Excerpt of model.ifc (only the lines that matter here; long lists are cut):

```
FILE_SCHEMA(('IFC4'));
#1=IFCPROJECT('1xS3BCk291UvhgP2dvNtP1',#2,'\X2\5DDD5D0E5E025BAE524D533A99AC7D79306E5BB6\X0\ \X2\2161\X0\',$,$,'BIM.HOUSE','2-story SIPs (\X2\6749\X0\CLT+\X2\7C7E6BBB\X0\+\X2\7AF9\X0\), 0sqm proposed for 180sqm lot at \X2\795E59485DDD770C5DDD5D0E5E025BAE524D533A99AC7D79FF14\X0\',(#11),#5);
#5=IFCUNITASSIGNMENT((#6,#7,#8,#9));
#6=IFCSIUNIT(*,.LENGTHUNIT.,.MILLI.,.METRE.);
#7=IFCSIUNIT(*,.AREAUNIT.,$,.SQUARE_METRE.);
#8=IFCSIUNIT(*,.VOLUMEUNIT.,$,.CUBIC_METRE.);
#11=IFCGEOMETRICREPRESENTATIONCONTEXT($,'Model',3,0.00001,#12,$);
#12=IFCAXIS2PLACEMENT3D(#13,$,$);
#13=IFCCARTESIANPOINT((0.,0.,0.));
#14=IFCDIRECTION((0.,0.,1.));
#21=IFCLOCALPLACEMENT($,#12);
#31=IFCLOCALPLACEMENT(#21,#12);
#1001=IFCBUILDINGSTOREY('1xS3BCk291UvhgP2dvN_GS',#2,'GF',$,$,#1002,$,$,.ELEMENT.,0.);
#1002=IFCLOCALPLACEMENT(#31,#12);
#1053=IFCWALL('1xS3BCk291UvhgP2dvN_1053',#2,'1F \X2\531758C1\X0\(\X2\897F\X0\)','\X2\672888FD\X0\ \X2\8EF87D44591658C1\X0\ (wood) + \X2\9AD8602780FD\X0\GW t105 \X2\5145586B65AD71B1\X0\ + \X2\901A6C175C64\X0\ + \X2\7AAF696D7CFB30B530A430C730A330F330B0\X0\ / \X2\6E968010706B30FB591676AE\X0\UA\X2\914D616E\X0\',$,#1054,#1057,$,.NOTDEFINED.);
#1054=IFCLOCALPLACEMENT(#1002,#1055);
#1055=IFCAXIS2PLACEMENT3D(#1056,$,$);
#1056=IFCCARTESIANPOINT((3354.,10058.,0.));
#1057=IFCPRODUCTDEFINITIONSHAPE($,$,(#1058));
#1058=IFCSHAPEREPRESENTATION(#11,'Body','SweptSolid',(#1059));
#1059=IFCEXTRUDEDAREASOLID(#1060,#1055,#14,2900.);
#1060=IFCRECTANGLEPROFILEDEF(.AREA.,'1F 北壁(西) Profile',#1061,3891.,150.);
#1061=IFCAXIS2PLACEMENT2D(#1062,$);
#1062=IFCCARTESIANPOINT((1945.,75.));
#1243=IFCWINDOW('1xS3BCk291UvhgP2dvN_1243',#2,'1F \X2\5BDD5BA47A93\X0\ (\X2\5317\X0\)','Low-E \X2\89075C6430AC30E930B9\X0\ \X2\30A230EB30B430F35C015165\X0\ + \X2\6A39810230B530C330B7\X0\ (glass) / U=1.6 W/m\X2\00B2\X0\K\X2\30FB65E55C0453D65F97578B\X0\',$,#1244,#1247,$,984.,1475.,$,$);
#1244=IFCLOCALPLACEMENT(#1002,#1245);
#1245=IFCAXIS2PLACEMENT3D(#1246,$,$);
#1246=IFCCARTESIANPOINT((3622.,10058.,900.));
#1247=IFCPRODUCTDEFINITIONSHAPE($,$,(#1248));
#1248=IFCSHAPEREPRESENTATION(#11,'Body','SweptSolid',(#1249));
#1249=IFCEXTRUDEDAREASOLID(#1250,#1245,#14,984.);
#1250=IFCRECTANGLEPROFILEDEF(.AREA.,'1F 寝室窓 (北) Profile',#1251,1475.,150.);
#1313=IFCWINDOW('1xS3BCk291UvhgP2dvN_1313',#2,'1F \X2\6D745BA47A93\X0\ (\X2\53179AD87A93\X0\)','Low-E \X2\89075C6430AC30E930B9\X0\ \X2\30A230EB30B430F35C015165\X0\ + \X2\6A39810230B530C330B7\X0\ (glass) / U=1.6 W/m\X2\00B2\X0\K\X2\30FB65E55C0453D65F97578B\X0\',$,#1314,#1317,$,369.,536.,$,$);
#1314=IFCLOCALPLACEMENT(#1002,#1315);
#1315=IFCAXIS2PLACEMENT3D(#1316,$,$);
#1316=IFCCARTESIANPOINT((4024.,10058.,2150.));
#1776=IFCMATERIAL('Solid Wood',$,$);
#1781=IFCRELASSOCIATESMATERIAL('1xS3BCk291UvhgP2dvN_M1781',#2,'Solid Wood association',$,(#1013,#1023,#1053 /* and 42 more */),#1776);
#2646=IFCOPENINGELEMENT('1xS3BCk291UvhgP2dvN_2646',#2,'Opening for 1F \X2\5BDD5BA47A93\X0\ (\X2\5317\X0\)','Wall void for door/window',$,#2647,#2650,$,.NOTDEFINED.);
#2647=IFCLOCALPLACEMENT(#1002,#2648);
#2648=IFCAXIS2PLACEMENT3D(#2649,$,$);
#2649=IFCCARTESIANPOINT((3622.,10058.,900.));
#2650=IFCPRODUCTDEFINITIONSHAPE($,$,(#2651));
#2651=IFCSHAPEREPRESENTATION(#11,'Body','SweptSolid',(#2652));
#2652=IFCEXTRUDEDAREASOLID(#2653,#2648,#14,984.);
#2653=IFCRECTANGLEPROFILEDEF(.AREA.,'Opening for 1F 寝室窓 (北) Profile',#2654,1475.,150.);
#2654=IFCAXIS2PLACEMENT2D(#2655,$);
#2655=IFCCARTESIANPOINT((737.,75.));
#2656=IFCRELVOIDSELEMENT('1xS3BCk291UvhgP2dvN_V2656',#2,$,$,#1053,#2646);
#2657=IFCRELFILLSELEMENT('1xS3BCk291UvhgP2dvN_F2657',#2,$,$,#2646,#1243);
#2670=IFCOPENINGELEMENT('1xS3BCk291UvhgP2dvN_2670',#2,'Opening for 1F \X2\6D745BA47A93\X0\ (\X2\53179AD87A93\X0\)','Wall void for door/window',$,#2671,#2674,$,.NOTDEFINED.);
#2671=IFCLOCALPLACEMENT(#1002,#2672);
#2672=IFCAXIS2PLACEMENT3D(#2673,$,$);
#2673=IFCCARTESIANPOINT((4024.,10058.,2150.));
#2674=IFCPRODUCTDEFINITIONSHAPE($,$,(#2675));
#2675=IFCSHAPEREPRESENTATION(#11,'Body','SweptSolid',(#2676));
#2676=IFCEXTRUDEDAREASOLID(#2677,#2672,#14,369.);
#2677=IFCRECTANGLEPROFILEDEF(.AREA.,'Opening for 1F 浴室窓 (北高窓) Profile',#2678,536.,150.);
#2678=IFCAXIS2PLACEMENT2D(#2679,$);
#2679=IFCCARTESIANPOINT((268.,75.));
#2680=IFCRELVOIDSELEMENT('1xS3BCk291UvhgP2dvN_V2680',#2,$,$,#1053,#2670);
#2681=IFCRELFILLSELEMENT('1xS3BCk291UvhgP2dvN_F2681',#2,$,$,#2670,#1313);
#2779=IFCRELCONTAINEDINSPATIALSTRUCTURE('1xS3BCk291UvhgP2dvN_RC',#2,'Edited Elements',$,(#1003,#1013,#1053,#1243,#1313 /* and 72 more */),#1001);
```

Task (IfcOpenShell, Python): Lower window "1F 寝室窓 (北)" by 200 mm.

```python
import numpy as np
import ifcopenshell
import ifcopenshell.api.geometry
import ifcopenshell.util.placement
import ifcopenshell.util.unit

model = ifcopenshell.open("model.ifc")
unit_scale = ifcopenshell.util.unit.calculate_unit_scale(model)

window = model.by_guid("1xS3BCk291UvhgP2dvN_1243")
opening = window.FillsVoids[0].RelatingOpeningElement
dz = -200.0

shift = np.array([0.0, 0.0, dz])
# The window is not placed relative to its opening, so move both.
for product in (opening, window):
    matrix = ifcopenshell.util.placement.get_local_placement(product.ObjectPlacement)
    matrix[:3, 3] += shift
    ifcopenshell.api.geometry.edit_object_placement(model, product=product, matrix=matrix, is_si=False)

print(f"moved by {dz * unit_scale:+.3f} m")

model.write("model_edited.ifc")
```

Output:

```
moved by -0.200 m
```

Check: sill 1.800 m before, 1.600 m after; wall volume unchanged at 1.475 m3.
